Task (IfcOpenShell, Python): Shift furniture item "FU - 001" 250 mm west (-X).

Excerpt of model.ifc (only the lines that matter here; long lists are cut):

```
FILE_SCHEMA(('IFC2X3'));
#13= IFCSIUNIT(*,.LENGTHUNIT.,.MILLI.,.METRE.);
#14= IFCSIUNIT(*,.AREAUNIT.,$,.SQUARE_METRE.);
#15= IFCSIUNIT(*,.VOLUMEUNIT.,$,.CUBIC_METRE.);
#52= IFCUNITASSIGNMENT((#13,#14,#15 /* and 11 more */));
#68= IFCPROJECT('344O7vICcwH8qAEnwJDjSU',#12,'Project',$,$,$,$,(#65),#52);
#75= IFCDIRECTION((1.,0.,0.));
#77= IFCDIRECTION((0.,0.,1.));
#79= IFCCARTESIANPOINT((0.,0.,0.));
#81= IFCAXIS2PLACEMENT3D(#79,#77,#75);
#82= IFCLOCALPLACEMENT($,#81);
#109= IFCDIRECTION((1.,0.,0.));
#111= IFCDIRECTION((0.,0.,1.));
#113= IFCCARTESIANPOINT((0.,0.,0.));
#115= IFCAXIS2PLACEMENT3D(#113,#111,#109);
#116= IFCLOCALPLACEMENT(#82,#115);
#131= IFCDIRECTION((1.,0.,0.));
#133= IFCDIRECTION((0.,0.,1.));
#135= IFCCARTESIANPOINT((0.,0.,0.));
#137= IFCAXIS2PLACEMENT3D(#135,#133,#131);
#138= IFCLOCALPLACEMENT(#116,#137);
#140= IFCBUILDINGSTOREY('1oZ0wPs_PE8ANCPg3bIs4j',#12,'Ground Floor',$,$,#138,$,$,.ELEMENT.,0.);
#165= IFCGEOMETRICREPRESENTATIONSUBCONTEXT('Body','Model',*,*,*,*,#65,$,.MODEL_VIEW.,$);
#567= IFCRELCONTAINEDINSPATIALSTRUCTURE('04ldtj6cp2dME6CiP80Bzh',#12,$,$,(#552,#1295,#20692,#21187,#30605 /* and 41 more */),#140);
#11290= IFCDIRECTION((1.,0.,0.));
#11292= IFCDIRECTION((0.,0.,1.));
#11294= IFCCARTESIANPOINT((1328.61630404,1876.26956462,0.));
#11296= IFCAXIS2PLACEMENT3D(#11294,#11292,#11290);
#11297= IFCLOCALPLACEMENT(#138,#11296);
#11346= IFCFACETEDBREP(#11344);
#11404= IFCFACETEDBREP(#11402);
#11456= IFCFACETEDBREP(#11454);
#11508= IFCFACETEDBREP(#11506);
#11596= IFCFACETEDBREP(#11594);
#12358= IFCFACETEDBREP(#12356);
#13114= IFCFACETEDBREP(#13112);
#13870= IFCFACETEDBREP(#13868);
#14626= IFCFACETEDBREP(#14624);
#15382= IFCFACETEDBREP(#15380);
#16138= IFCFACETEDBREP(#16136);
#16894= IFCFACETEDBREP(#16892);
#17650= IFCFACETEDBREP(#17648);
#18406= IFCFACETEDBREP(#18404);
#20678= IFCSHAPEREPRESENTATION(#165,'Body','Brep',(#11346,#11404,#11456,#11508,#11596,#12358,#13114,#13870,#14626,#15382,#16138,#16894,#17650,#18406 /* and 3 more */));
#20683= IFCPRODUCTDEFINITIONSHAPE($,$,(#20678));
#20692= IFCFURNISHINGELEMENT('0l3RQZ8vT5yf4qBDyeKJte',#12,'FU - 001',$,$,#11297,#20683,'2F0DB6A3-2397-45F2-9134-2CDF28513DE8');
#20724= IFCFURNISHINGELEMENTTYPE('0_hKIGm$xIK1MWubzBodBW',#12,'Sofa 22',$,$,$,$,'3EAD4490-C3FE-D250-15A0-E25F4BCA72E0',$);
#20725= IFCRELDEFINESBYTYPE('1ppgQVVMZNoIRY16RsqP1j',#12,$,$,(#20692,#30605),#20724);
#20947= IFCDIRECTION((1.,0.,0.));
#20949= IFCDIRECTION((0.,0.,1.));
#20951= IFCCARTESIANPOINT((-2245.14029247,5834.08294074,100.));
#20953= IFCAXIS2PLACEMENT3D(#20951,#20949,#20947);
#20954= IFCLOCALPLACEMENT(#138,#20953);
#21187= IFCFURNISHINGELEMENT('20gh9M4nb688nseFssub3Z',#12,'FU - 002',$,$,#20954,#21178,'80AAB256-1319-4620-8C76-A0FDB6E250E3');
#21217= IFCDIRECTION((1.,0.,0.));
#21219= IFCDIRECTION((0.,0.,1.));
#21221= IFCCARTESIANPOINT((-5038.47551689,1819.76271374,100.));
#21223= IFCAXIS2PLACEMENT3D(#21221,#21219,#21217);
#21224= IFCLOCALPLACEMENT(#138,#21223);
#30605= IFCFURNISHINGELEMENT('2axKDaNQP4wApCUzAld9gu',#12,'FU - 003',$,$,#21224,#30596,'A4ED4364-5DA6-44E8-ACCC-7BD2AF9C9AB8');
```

```python
import ifcopenshell
import ifcopenshell.api.geometry
import ifcopenshell.util.placement
import ifcopenshell.util.unit

model = ifcopenshell.open("model.ifc")
unit_scale = ifcopenshell.util.unit.calculate_unit_scale(model)

item = model.by_guid("0l3RQZ8vT5yf4qBDyeKJte")
matrix = ifcopenshell.util.placement.get_local_placement(item.ObjectPlacement)
matrix[0, 3] -= 0.25 / unit_scale
ifcopenshell.api.geometry.edit_object_placement(model, product=item, matrix=matrix, is_si=False)

print(ifcopenshell.util.placement.get_local_placement(item.ObjectPlacement).round(3) + 0.0)

model.write("model_v2.ifc")
```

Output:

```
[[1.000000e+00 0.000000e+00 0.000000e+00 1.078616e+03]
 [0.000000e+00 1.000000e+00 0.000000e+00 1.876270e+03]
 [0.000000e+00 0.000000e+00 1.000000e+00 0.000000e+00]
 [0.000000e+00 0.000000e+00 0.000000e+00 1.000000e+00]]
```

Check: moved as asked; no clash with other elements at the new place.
